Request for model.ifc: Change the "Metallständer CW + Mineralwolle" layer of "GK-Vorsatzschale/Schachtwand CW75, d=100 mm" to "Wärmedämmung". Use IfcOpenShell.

First a look at what the model holds.

```python
import ifcopenshell
import ifcopenshell.util.element

model = ifcopenshell.open("model.ifc")
print(model.schema)
for layer_set in model.by_type("IfcMaterialLayerSet"):
    if layer_set.LayerSetName == "GK-Vorsatzschale/Schachtwand CW75, d=100 mm":
        for layer in layer_set.MaterialLayers:
            print(layer.id(), layer.Material and layer.Material.Name, layer.LayerThickness, sep=" | ")
        print(len(ifcopenshell.util.element.get_elements_by_material(model, layer_set)), "elements and types use it")
print(sorted(m.Name for m in model.by_type("IfcMaterial") if m.Name)[:60])
```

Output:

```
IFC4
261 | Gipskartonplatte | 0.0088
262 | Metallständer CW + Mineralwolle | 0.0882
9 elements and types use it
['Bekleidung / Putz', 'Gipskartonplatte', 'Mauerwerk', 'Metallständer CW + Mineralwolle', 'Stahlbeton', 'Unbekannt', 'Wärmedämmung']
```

```python
import ifcopenshell
import ifcopenshell.api.material

model = ifcopenshell.open("model.ifc")

layer_set = next(s for s in model.by_type("IfcMaterialLayerSet") if s.LayerSetName == "GK-Vorsatzschale/Schachtwand CW75, d=100 mm")
layer = next(l for l in layer_set.MaterialLayers if l.Material and l.Material.Name == "Metallständer CW + Mineralwolle")
material = next(m for m in model.by_type("IfcMaterial") if m.Name == "Wärmedämmung")

# Point this one layer at the other material; renaming the old one would change it everywhere.
ifcopenshell.api.material.edit_layer(model, layer=layer, attributes={"Name": material.Name}, material=material)

print([l.Material.Name if l.Material else None for l in layer_set.MaterialLayers])

model.write("model-out.ifc")
```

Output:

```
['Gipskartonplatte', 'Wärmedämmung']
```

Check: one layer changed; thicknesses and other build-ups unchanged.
